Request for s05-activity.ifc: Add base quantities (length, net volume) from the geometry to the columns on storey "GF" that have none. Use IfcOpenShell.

First a look at what the model holds.

```python
import ifcopenshell
import ifcopenshell.util.element
import ifcopenshell.util.unit

model = ifcopenshell.open("s05-activity.ifc")
print(model.schema)
for unit_type in ("LENGTHUNIT", "AREAUNIT", "VOLUMEUNIT"):
    print(unit_type, ifcopenshell.util.unit.calculate_unit_scale(model, unit_type))
storey = next(s for s in model.by_type("IfcBuildingStorey") if s.Name == "GF")
columns = [e for e in ifcopenshell.util.element.get_decomposition(storey) if e.is_a("IfcColumn")]
for e in sorted(columns, key=lambda e: e.id()):
    print(e.id(), e.is_a(), e.Name, list(ifcopenshell.util.element.get_psets(e, qtos_only=True)), sep=" | ")
```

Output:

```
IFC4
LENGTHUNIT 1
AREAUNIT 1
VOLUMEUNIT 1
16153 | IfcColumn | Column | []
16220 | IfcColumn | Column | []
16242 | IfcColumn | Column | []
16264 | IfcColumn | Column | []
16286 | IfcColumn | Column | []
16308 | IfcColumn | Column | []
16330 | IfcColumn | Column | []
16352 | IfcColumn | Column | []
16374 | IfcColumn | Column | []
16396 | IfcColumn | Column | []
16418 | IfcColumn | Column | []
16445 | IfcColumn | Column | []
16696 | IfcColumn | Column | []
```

```python
import ifcopenshell
import ifcopenshell.api.pset
import ifcopenshell.geom
import ifcopenshell.util.element
import ifcopenshell.util.shape
import ifcopenshell.util.unit

model = ifcopenshell.open("s05-activity.ifc")
unit_scale = ifcopenshell.util.unit.calculate_unit_scale(model)
volume_scale = ifcopenshell.util.unit.calculate_unit_scale(model, "VOLUMEUNIT")
settings = ifcopenshell.geom.settings()

storey = next(s for s in model.by_type("IfcBuildingStorey") if s.Name == "GF")
columns = [e for e in ifcopenshell.util.element.get_decomposition(storey) if e.is_a("IfcColumn")]

for e in sorted(columns, key=lambda e: e.id()):
    if ifcopenshell.util.element.get_psets(e, qtos_only=True, should_inherit=False):
        continue
    # Geometry comes back in metres, in the element's own axes.
    shape = ifcopenshell.geom.create_shape(settings, e)
    values = {
        "Length": ifcopenshell.util.shape.get_z(shape.geometry) / unit_scale,
        "NetVolume": ifcopenshell.util.shape.get_volume(shape.geometry) / volume_scale,
    }
    qto = ifcopenshell.api.pset.add_qto(model, product=e, name="Qto_ColumnBaseQuantities")
    ifcopenshell.api.pset.edit_qto(model, qto=qto, properties=values)
    print(e.id(), {k: round(v, 3) for k, v in values.items()})

model.write("s05-activity-out.ifc")
```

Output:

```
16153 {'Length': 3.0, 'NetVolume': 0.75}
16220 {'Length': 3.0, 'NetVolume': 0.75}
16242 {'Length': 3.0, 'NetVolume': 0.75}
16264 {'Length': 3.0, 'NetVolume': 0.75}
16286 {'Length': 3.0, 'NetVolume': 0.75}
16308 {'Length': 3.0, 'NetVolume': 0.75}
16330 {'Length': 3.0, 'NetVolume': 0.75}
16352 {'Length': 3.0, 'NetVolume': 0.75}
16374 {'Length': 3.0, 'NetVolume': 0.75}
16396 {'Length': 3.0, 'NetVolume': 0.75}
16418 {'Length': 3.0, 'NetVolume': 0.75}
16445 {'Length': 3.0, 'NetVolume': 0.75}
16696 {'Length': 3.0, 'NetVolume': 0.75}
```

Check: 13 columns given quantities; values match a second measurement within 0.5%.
